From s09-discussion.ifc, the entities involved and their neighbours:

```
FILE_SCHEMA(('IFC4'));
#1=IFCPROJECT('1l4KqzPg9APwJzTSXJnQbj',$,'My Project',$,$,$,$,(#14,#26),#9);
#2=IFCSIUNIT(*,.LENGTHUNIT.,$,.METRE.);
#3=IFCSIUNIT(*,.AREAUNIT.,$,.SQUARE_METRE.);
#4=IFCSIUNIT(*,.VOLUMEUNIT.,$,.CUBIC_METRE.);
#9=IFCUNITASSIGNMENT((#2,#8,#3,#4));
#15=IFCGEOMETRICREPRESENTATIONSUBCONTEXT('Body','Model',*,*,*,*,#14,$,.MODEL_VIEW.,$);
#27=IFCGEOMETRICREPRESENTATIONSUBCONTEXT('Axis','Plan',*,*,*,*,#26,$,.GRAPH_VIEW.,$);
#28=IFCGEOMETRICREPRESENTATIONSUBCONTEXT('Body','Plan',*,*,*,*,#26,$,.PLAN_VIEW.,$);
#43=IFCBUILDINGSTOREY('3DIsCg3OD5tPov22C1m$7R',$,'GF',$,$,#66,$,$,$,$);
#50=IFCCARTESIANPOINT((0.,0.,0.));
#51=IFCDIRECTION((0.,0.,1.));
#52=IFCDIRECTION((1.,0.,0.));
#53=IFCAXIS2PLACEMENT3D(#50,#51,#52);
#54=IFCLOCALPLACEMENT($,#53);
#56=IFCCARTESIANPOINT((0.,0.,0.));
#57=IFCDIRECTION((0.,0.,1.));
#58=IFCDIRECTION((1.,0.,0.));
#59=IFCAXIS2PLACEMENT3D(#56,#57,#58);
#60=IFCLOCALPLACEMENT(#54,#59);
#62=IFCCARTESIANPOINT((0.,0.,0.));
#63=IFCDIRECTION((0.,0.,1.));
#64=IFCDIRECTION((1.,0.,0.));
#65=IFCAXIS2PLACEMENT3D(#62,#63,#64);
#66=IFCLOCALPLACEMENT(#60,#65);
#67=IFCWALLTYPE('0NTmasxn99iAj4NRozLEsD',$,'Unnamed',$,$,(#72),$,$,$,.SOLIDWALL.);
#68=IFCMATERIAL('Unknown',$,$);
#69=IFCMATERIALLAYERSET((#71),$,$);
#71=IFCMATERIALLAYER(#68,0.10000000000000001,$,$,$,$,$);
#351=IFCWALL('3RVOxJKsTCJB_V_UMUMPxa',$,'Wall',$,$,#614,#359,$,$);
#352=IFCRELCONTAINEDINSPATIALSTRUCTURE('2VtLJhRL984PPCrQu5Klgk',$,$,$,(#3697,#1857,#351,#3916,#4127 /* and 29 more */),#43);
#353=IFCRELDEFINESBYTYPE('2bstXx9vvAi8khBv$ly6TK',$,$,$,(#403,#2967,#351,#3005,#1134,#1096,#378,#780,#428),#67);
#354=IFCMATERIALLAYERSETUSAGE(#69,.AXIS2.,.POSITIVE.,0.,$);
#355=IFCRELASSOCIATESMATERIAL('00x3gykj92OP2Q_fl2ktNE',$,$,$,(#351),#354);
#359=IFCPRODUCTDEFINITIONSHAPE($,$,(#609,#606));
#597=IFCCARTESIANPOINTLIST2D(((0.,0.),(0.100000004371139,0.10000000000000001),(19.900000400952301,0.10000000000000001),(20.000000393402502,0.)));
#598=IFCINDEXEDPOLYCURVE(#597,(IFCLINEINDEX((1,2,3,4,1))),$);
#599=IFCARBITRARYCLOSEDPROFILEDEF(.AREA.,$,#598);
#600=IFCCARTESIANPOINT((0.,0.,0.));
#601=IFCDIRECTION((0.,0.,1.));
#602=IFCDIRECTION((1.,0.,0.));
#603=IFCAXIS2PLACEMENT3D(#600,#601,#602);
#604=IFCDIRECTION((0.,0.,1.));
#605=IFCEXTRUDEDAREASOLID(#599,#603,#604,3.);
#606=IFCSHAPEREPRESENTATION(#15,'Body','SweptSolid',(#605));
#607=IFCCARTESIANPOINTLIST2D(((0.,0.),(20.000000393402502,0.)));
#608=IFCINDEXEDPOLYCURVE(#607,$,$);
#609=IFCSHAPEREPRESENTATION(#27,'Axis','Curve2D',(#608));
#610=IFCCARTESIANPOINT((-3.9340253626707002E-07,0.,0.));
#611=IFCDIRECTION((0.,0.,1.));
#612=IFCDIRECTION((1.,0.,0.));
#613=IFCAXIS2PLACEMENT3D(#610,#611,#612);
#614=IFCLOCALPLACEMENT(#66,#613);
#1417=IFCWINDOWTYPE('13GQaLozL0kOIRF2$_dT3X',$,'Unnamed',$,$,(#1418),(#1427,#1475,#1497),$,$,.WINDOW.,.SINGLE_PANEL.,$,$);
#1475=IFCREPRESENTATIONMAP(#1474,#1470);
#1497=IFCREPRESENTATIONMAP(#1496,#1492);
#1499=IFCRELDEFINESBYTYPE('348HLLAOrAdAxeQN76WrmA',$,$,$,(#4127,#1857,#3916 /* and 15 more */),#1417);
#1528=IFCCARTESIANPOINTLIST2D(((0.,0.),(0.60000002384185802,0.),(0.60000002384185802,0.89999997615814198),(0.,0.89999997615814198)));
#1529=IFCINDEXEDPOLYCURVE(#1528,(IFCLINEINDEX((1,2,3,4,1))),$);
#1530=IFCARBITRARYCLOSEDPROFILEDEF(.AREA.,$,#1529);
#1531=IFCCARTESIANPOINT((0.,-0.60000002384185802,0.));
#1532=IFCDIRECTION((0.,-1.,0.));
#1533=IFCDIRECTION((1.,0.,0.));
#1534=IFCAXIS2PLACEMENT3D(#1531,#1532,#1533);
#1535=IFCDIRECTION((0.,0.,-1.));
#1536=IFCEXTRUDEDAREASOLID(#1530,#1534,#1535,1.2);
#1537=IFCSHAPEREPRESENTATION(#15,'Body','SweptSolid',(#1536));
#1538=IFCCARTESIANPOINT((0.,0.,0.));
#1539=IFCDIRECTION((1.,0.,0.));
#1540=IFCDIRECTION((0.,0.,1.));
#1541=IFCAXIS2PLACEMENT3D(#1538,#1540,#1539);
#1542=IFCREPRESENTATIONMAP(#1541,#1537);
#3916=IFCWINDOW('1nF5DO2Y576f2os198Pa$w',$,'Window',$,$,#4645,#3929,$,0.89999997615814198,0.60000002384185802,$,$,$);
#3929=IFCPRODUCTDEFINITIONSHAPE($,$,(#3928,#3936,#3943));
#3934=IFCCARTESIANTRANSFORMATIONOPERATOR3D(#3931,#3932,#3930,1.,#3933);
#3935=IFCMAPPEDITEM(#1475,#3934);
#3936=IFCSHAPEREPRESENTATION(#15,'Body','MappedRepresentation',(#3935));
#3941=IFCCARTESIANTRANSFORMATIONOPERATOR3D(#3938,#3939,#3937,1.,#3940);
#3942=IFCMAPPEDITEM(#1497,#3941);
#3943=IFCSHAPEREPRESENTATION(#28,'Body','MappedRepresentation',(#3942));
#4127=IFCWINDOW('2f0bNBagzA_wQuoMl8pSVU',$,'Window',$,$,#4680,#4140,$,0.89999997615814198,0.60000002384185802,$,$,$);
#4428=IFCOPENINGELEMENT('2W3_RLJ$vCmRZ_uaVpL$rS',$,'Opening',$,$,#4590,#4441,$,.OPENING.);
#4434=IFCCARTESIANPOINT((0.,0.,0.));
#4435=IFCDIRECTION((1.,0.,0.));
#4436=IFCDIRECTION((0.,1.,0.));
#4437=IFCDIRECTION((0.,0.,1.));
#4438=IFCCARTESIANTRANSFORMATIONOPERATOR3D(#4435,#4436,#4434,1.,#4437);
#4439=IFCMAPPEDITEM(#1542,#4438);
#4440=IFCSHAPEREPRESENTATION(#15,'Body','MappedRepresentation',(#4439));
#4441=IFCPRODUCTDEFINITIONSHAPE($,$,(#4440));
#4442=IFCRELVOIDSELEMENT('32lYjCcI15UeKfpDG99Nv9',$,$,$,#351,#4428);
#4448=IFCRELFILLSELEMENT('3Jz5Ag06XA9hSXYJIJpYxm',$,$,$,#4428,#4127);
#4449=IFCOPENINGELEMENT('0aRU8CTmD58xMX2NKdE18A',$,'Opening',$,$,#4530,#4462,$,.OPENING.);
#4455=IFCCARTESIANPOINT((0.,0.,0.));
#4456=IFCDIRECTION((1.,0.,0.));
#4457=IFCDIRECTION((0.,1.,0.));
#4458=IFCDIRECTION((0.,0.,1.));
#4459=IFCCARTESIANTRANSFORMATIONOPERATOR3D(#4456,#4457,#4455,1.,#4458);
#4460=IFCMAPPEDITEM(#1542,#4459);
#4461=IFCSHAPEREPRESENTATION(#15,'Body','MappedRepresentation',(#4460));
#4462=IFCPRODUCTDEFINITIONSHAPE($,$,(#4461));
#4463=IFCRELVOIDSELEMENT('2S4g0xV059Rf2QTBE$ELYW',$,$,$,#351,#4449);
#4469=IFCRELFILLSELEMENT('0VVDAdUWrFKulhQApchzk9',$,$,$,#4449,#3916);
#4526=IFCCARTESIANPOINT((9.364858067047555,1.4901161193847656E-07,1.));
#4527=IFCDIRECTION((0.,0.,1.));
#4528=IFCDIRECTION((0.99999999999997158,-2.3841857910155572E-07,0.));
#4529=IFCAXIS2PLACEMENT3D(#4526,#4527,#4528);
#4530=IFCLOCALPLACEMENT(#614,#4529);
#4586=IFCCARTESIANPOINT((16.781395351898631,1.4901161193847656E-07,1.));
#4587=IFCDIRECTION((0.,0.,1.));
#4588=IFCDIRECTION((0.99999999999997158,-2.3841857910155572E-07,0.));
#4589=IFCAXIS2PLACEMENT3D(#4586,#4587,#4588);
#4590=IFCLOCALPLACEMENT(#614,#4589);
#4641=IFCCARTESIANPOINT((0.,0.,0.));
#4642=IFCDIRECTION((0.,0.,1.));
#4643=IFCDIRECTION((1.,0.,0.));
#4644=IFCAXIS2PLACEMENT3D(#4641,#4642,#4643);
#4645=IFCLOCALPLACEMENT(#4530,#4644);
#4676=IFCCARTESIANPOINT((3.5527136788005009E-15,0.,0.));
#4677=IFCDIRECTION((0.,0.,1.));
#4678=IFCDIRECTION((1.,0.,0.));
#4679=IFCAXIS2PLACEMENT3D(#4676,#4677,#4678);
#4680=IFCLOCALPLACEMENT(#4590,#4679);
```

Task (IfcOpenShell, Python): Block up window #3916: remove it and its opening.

```python
import ifcopenshell
import ifcopenshell.api.feature
import ifcopenshell.api.root
import ifcopenshell.geom
import ifcopenshell.util.shape

model = ifcopenshell.open("s09-discussion.ifc")
settings = ifcopenshell.geom.settings()


def volume(element):
    """Net volume in cubic metres, openings subtracted."""
    shape = ifcopenshell.geom.create_shape(settings, element)
    return ifcopenshell.util.shape.get_volume(shape.geometry)


window = model.by_id(3916)
opening = window.FillsVoids[0].RelatingOpeningElement
wall = opening.VoidsElements[0].RelatingBuildingElement
before = volume(wall)

ifcopenshell.api.root.remove_product(model, product=window)
ifcopenshell.api.feature.remove_feature(model, feature=opening)

after = volume(wall)

print(f"wall volume {before:.3f} -> {after:.3f} m3")

model.write("s09-discussion_updated.ifc")
```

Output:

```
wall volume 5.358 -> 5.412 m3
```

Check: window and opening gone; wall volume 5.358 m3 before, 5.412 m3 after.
